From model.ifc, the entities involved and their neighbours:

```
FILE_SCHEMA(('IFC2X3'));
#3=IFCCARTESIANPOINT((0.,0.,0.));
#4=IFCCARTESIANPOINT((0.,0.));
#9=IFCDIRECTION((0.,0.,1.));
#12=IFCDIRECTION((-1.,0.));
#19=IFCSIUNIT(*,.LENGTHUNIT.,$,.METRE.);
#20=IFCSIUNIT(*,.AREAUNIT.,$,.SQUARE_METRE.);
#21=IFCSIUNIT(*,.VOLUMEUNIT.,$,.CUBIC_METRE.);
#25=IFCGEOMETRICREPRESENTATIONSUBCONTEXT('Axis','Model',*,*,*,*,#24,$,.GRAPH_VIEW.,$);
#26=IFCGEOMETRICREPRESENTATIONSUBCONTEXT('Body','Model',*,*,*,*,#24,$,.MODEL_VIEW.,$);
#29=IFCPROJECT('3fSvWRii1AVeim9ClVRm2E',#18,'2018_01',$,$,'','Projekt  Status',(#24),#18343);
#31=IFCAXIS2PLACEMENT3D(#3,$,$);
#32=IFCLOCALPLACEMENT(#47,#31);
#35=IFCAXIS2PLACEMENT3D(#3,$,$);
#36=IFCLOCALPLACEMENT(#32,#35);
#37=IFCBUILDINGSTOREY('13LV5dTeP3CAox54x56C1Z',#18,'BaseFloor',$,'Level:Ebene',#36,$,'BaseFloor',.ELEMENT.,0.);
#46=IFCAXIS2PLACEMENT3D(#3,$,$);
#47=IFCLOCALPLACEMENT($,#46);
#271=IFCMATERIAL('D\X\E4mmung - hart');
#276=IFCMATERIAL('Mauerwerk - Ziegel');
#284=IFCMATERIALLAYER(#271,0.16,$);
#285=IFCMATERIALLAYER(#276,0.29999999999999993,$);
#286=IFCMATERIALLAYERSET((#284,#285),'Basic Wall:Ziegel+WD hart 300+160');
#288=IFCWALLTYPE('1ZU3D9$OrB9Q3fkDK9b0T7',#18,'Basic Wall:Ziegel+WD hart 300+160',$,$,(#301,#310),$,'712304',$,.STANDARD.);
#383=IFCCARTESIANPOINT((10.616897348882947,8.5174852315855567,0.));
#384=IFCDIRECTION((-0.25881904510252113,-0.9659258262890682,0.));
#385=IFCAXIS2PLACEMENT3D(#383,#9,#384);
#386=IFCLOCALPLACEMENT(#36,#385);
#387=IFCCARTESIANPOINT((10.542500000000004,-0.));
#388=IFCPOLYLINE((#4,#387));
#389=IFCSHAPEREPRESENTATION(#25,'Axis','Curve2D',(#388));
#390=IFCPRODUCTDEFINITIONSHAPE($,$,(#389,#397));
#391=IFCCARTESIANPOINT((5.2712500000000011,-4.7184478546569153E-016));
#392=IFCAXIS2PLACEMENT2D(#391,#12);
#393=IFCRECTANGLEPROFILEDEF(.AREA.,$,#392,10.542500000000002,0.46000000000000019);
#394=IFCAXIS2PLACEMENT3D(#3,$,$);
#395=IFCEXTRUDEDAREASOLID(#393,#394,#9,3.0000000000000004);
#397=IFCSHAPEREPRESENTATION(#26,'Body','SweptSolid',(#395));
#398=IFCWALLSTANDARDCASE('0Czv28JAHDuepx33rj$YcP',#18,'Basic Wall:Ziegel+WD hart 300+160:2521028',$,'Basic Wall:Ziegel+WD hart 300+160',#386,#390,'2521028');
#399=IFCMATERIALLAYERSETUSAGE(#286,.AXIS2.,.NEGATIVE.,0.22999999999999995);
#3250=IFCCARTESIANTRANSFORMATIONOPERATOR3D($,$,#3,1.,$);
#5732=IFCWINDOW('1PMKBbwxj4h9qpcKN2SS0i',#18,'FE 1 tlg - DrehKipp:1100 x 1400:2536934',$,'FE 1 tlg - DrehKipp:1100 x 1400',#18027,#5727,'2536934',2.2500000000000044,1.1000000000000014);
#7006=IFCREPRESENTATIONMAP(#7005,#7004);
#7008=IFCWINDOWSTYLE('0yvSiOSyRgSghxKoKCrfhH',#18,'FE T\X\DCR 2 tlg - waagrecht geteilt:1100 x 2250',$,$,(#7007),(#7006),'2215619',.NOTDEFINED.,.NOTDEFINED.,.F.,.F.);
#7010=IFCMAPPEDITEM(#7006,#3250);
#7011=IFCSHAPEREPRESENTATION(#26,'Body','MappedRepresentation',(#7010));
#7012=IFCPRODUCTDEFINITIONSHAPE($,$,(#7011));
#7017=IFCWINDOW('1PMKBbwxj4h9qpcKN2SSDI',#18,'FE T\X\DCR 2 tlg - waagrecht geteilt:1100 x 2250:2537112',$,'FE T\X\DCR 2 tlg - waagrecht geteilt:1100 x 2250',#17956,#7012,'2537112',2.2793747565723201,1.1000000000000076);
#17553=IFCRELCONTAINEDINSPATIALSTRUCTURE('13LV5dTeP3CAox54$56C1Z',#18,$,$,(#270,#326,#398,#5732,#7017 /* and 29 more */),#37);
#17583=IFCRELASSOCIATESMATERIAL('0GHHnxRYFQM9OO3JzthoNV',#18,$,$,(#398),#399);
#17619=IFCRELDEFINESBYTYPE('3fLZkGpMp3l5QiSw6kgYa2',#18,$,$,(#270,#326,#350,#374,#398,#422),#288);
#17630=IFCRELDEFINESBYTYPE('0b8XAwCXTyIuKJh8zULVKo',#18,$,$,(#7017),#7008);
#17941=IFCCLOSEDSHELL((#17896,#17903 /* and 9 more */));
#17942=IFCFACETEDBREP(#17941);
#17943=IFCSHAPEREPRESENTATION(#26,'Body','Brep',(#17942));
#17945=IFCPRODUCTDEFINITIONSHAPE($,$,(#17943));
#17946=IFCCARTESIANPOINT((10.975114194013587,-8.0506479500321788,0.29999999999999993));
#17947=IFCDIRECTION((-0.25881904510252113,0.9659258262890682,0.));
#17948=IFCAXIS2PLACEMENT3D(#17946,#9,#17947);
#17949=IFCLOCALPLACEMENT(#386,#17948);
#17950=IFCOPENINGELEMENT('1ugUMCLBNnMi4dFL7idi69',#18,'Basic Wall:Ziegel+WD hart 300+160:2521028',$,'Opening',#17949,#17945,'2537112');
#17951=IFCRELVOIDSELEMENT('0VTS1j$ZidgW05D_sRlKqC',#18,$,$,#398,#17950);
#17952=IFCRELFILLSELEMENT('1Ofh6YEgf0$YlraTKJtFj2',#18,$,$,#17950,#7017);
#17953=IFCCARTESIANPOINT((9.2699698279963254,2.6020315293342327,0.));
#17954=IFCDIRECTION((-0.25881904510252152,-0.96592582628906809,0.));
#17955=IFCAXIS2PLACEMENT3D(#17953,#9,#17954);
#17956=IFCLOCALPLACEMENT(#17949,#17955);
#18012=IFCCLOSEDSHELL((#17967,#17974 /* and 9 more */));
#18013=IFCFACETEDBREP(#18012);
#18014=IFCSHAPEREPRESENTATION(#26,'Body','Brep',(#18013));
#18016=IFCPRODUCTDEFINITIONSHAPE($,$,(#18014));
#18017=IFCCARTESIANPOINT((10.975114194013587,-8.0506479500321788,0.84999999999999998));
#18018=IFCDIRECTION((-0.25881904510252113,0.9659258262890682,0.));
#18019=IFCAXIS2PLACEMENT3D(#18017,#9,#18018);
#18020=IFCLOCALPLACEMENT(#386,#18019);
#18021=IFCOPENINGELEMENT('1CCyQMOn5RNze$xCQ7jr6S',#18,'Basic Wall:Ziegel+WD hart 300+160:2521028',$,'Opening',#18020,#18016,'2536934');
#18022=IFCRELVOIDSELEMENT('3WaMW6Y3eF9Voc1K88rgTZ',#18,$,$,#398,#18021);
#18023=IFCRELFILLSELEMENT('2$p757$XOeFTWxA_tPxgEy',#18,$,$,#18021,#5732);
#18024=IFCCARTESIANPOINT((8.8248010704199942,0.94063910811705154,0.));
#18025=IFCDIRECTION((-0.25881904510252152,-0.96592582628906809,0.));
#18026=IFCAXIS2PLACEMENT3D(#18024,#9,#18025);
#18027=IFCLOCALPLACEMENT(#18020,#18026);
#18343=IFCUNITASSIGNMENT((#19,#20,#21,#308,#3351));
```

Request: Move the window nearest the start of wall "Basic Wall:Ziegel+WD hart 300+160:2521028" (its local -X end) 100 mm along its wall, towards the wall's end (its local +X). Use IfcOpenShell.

```python
import ifcopenshell
import ifcopenshell.api.geometry
import ifcopenshell.util.placement

model = ifcopenshell.open("model.ifc")

window = model.by_guid("1PMKBbwxj4h9qpcKN2SSDI")
opening = window.FillsVoids[0].RelatingOpeningElement
wall = opening.VoidsElements[0].RelatingBuildingElement

wall_matrix = ifcopenshell.util.placement.get_local_placement(wall.ObjectPlacement)
shift = wall_matrix[:3, 0] * 0.1
before = ifcopenshell.util.placement.get_local_placement(window.ObjectPlacement)[:3, 3].copy()

# The window is placed relative to its opening, so it follows when the opening moves.
matrix = ifcopenshell.util.placement.get_local_placement(opening.ObjectPlacement)
matrix[:3, 3] += shift
ifcopenshell.api.geometry.edit_object_placement(
    model, product=opening, matrix=matrix, is_si=False, should_transform_children=True
)

after = ifcopenshell.util.placement.get_local_placement(window.ObjectPlacement)[:3, 3]
print("window moved by", (after - before).round(3) + 0.0)

model.write("model_v2.ifc")
```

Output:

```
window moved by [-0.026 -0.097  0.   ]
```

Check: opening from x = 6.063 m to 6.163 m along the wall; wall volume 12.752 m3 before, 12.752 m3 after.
